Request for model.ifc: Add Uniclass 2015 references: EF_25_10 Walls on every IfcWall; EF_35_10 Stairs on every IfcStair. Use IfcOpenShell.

First a look at what the model holds.

```python
import ifcopenshell

model = ifcopenshell.open("model.ifc")
print(model.schema)
print("classifications:", [c.Name for c in model.by_type("IfcClassification")])
for ifc_class in ("IfcDoor", "IfcRoof", "IfcStair", "IfcWall", "IfcWindow"):
    print(ifc_class, len(model.by_type(ifc_class)))
```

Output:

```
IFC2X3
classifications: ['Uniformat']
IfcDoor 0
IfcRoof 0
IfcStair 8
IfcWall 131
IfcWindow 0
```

```python
import ifcopenshell
import ifcopenshell.api.classification

model = ifcopenshell.open("model.ifc")

# IFC2X3 requires Source and Edition and has no link from the project to the system.
system = model.create_entity("IfcClassification", Source="NBS", Edition="2015", Name="Uniclass 2015")

codes = {
    "IfcWall": ("EF_25_10", "Walls"),
    "IfcStair": ("EF_35_10", "Stairs"),
}
for ifc_class, (code, name) in codes.items():
    products = model.by_type(ifc_class)
    ifcopenshell.api.classification.add_reference(
        model, products=products, classification=system, identification=code, name=name
    )
    print(code, len(products))

model.write("model_edited.ifc")
```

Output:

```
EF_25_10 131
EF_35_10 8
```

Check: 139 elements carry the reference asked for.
